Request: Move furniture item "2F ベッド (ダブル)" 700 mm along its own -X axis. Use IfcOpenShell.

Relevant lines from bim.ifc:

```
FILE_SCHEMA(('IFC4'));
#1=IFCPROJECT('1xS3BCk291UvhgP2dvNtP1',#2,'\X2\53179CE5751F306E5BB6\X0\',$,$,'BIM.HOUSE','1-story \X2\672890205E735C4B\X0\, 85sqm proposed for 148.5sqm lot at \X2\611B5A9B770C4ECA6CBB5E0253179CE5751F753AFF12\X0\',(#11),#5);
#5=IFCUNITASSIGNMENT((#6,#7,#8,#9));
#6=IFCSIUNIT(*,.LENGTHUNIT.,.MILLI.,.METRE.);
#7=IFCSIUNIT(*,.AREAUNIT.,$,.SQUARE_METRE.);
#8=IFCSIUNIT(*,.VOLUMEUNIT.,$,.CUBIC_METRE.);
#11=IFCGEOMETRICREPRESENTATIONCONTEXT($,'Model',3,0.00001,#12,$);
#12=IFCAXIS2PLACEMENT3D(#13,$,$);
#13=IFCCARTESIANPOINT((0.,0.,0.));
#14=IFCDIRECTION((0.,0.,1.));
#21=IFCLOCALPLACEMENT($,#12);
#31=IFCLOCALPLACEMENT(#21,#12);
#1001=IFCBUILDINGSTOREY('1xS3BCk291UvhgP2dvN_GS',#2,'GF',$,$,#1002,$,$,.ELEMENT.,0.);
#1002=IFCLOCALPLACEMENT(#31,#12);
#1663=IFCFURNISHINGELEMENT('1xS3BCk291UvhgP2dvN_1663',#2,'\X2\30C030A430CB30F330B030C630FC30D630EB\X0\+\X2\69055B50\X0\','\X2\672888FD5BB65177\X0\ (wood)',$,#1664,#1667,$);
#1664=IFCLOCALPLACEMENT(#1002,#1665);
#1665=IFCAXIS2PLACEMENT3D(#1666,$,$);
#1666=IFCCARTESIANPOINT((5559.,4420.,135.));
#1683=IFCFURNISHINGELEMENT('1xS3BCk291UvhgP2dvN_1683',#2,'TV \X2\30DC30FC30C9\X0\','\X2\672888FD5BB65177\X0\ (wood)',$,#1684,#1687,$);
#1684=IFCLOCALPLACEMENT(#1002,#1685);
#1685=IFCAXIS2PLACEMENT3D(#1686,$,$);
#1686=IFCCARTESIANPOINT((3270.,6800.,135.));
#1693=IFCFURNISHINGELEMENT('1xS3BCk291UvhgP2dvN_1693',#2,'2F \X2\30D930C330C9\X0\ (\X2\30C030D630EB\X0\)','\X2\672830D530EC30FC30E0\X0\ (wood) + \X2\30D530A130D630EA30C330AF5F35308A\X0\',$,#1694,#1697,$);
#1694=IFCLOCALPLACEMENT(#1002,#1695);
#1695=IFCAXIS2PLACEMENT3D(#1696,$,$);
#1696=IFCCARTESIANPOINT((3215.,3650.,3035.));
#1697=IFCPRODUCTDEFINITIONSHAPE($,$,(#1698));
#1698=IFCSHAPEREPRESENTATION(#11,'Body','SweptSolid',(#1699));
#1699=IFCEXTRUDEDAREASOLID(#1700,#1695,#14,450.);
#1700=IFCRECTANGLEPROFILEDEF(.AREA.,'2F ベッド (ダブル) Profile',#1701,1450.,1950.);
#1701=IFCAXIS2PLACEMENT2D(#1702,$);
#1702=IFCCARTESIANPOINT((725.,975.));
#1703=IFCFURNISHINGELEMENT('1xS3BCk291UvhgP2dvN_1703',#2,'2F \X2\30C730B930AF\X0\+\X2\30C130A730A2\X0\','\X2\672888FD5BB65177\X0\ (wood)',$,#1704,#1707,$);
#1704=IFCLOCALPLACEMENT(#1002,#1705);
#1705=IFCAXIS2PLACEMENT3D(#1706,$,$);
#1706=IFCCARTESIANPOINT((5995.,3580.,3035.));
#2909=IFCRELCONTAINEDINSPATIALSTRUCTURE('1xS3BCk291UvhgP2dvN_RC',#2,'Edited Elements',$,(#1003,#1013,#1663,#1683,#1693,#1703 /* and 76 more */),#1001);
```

```python
import ifcopenshell
import ifcopenshell.api.geometry
import ifcopenshell.util.placement
import ifcopenshell.util.unit

model = ifcopenshell.open("bim.ifc")
unit_scale = ifcopenshell.util.unit.calculate_unit_scale(model)

item = model.by_guid("1xS3BCk291UvhgP2dvN_1693")
matrix = ifcopenshell.util.placement.get_local_placement(item.ObjectPlacement)
matrix[:3, 3] -= matrix[:3, 0] * 0.7 / unit_scale
ifcopenshell.api.geometry.edit_object_placement(model, product=item, matrix=matrix, is_si=False)

print(ifcopenshell.util.placement.get_local_placement(item.ObjectPlacement).round(3) + 0.0)

model.write("bim_rev.ifc")
```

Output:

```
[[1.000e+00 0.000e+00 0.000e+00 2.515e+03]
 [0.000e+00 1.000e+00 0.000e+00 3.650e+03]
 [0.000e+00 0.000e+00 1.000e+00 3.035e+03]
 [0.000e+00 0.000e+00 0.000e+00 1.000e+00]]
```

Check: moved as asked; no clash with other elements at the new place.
